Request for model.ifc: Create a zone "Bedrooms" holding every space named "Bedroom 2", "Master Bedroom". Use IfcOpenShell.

First a look at what the model holds.

```python
import ifcopenshell

model = ifcopenshell.open("model.ifc")
print(model.schema)
seen = {}
for space in model.by_type("IfcSpace"):
    seen[space.LongName] = seen.get(space.LongName, 0) + 1
for name, count in sorted(seen.items(), key=str):
    print(count, "x", name)
print("zones:", [z.Name for z in model.by_type("IfcZone")][:20])
```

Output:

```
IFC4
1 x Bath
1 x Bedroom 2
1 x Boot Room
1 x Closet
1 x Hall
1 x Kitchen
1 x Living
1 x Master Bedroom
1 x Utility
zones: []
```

```python
import ifcopenshell
import ifcopenshell.api.group
import ifcopenshell.api.root

model = ifcopenshell.open("model.ifc")

names = {"Bedroom 2", "Master Bedroom"}
spaces = [s for s in model.by_type("IfcSpace") if s.LongName in names]

zone = ifcopenshell.api.root.create_entity(model, ifc_class="IfcZone", name="Bedrooms")
ifcopenshell.api.group.assign_group(model, products=spaces, group=zone)
print(len(spaces), "spaces in", zone.Name)

model.write("model_updated.ifc")
```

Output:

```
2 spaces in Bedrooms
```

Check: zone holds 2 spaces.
